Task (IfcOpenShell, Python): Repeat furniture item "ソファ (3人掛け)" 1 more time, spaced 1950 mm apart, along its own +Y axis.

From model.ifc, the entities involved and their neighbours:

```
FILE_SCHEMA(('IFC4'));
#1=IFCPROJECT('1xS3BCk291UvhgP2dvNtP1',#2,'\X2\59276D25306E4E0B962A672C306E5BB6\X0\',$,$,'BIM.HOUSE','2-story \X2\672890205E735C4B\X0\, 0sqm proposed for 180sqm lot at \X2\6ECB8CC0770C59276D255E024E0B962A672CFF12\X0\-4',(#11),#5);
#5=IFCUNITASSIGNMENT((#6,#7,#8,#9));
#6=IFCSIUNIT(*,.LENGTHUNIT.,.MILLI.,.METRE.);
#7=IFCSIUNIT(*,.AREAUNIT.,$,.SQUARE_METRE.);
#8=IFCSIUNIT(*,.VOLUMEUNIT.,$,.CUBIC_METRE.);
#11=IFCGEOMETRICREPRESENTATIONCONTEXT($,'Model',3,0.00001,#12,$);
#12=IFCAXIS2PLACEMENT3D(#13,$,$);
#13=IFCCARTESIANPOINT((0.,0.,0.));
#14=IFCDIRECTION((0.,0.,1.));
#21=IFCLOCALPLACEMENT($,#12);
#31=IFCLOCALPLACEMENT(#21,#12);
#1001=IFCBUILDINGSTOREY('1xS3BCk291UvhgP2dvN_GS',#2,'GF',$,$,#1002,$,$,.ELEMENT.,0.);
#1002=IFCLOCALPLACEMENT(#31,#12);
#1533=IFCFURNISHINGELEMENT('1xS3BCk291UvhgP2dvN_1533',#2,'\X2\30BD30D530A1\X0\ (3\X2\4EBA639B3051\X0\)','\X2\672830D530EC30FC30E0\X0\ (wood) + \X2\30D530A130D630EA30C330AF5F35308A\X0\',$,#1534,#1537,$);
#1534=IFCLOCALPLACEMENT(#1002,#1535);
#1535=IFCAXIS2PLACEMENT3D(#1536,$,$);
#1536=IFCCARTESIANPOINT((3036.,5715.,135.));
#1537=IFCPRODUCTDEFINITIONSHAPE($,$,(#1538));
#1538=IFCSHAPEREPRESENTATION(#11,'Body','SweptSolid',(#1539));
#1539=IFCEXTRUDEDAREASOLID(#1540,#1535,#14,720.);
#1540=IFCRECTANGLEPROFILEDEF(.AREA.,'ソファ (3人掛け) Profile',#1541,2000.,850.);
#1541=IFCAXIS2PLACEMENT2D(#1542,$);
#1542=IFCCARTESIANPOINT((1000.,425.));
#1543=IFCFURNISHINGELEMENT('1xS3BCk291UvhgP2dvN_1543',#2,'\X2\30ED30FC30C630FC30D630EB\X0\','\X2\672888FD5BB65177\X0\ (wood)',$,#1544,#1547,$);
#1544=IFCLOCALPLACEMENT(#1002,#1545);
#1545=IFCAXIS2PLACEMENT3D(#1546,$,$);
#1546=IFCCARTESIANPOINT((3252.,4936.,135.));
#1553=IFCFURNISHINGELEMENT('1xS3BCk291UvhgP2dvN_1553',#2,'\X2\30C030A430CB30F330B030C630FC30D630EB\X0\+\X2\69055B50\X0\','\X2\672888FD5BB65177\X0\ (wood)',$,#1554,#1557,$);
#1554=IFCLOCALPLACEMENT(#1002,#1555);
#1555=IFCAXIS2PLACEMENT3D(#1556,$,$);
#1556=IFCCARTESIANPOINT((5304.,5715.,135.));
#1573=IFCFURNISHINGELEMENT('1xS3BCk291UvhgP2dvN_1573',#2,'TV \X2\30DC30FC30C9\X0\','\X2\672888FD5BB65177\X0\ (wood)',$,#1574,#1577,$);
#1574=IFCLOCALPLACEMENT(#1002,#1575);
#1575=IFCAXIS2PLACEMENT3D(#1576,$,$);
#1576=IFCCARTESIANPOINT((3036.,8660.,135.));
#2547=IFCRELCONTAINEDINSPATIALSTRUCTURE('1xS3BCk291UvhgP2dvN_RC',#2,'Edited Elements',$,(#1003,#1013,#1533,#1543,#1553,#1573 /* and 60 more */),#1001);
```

```python
import ifcopenshell
import ifcopenshell.api.geometry
import ifcopenshell.api.root
import ifcopenshell.util.element
import ifcopenshell.util.placement
import ifcopenshell.util.unit

model = ifcopenshell.open("model.ifc")
unit_scale = ifcopenshell.util.unit.calculate_unit_scale(model)


def reuse_history(source, copy):
    """copy_class also copies each property set's owner history, people and application; keep the originals."""
    for rel in copy.IsDefinedBy:
        if rel.is_a("IfcRelDefinesByProperties") and (history := rel.RelatingPropertyDefinition.OwnerHistory):
            rel.RelatingPropertyDefinition.OwnerHistory = source.OwnerHistory
            ifcopenshell.util.element.remove_deep2(model, history)


source = model.by_guid("1xS3BCk291UvhgP2dvN_1533")
base = ifcopenshell.util.placement.get_local_placement(source.ObjectPlacement)
step = base[:3, 1] * 1.95 / unit_scale

for i in range(1, 2):
    copy = ifcopenshell.api.root.copy_class(model, product=source)
    copy.Representation = ifcopenshell.util.element.copy_deep(
        model, source.Representation, exclude=["IfcGeometricRepresentationContext", "IfcRepresentationMap"]
    )
    reuse_history(source, copy)
    matrix = base.copy()
    matrix[:3, 3] += i * step
    print("added at", matrix[:3, 3].round(3) + 0.0)
    ifcopenshell.api.geometry.edit_object_placement(model, product=copy, matrix=matrix, is_si=False)

model.write("model_v2.ifc")
```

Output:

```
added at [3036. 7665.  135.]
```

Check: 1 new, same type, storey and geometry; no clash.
